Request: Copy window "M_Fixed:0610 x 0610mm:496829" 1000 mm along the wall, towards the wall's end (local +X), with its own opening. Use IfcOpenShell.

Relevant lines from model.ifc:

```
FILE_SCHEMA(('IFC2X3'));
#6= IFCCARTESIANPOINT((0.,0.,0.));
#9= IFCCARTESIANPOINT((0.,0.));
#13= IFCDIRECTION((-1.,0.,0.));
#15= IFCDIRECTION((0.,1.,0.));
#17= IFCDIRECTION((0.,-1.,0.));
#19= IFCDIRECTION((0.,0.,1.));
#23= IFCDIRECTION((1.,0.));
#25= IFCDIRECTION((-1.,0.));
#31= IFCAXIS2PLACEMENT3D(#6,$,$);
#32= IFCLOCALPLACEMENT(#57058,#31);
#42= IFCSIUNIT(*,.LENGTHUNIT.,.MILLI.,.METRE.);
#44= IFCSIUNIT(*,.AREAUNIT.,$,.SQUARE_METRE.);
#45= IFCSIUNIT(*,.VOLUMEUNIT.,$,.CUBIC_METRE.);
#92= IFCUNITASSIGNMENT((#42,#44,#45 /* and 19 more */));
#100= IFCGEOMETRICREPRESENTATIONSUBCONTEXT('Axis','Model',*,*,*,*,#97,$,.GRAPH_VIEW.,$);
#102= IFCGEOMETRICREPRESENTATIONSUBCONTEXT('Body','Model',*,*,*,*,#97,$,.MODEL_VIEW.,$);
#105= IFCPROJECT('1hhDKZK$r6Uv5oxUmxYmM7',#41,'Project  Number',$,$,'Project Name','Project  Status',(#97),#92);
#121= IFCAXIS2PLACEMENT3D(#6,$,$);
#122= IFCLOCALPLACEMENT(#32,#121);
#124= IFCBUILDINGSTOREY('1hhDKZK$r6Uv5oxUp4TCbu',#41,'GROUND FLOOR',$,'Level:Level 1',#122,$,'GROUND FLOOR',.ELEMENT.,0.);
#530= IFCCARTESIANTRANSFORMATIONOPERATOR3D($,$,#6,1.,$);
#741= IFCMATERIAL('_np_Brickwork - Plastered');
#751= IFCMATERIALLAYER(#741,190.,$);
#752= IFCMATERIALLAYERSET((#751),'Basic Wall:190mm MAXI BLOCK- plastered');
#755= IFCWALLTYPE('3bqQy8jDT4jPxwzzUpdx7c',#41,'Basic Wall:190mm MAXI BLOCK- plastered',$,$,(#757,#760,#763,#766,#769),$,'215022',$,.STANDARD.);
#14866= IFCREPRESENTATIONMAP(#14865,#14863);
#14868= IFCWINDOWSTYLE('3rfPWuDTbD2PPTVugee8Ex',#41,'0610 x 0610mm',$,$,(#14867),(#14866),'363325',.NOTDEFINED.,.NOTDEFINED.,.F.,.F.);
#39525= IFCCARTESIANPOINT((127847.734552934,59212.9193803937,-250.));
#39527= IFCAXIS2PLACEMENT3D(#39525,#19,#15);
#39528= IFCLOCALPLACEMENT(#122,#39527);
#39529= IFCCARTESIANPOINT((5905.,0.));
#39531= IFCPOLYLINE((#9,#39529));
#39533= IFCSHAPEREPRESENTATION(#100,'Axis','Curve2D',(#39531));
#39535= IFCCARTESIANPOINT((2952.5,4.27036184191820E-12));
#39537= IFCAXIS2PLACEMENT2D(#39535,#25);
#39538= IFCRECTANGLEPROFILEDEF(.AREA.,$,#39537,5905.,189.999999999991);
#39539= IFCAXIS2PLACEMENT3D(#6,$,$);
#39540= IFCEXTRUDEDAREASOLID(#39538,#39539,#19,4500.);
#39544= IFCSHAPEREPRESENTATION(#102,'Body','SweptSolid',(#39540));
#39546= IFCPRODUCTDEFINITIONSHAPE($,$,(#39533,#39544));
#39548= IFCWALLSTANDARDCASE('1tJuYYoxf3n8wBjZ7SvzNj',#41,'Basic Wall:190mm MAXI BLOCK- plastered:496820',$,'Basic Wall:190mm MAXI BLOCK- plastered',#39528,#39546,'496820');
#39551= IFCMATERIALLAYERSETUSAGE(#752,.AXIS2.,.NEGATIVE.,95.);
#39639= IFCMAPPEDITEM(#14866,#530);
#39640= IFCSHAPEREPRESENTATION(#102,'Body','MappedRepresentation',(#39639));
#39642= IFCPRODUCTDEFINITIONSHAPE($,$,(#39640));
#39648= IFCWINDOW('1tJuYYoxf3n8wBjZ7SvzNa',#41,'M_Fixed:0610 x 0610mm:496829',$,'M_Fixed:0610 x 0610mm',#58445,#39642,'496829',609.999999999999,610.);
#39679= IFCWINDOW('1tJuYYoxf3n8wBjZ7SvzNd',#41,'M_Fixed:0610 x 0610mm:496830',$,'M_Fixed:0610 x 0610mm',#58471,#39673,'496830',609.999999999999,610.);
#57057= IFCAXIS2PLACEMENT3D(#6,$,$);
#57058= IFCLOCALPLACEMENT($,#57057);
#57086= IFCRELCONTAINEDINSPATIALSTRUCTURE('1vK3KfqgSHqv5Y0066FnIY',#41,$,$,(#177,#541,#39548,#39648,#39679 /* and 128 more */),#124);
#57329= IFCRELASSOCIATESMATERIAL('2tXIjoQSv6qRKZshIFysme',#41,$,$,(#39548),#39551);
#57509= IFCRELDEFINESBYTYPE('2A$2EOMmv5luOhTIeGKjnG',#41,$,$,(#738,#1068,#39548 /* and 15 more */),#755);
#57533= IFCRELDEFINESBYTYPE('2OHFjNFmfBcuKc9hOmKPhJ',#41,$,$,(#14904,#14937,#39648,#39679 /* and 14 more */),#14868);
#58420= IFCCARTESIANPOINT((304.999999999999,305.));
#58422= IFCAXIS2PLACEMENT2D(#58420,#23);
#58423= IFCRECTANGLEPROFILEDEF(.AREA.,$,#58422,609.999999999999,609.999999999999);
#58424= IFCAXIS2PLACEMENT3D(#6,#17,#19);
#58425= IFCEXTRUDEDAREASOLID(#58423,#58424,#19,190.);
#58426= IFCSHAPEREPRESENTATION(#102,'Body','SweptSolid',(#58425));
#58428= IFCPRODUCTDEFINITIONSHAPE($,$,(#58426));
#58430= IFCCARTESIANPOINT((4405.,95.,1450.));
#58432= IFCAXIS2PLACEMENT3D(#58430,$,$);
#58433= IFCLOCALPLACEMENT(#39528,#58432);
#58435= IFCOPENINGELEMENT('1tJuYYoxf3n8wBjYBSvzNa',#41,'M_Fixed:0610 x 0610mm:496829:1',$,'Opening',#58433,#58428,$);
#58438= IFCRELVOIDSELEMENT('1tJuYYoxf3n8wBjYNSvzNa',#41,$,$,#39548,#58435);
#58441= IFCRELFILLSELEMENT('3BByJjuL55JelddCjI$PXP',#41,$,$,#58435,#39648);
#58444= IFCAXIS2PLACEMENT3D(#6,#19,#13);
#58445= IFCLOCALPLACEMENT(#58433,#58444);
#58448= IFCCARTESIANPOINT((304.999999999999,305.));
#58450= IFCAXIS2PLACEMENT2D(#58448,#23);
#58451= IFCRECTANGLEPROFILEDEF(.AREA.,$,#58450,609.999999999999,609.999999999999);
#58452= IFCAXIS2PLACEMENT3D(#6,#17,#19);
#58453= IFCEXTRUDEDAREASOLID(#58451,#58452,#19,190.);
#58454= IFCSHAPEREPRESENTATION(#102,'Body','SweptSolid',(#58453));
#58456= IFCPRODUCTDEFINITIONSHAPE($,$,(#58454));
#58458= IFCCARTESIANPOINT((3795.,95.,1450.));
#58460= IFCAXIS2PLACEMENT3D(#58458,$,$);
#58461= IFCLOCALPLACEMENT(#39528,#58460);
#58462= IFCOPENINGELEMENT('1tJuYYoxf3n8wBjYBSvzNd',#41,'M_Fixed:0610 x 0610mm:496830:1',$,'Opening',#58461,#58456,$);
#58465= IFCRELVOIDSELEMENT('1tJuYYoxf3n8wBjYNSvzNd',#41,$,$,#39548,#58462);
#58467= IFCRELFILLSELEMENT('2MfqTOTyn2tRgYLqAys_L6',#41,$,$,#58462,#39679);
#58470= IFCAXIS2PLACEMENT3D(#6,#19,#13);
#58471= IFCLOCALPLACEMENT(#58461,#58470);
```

```python
import ifcopenshell
import ifcopenshell.api.feature
import ifcopenshell.api.geometry
import ifcopenshell.api.root
import ifcopenshell.geom
import ifcopenshell.util.element
import ifcopenshell.util.placement
import ifcopenshell.util.shape
import ifcopenshell.util.unit

model = ifcopenshell.open("model.ifc")
unit_scale = ifcopenshell.util.unit.calculate_unit_scale(model)
settings = ifcopenshell.geom.settings()


def volume(element):
    """Net volume in cubic metres, openings subtracted."""
    shape = ifcopenshell.geom.create_shape(settings, element)
    return ifcopenshell.util.shape.get_volume(shape.geometry)


def reuse_history(source, copy):
    """copy_class also copies each property set's owner history, people and application; keep the originals."""
    for rel in copy.IsDefinedBy:
        if rel.is_a("IfcRelDefinesByProperties") and (history := rel.RelatingPropertyDefinition.OwnerHistory):
            rel.RelatingPropertyDefinition.OwnerHistory = source.OwnerHistory
            ifcopenshell.util.element.remove_deep2(model, history)


window = model.by_guid("1tJuYYoxf3n8wBjZ7SvzNa")
opening = window.FillsVoids[0].RelatingOpeningElement
wall = opening.VoidsElements[0].RelatingBuildingElement
before = volume(wall)
shift = ifcopenshell.util.placement.get_local_placement(wall.ObjectPlacement)[:3, 0] * 1 / unit_scale

# copy_class copies the void relationship, type, container and properties, but no geometry.
new_opening = ifcopenshell.api.root.copy_class(model, product=opening)
new_opening.Representation = ifcopenshell.util.element.copy_deep(
    model, opening.Representation, exclude=["IfcGeometricRepresentationContext", "IfcRepresentationMap"]
)
new_opening.Name = "M_Fixed:0610 x 0610mm"
new_window = ifcopenshell.api.root.copy_class(model, product=window)
new_window.Representation = ifcopenshell.util.element.copy_deep(
    model, window.Representation, exclude=["IfcGeometricRepresentationContext", "IfcRepresentationMap"]
)
new_window.Name = "M_Fixed:0610 x 0610mm"
new_window.Tag = None
reuse_history(window, new_window)
fills = ifcopenshell.api.feature.add_filling(model, opening=new_opening, element=new_window)
fills.OwnerHistory = new_window.OwnerHistory  # required in IFC2X3

for old, new in ((opening, new_opening), (window, new_window)):
    matrix = ifcopenshell.util.placement.get_local_placement(old.ObjectPlacement)
    matrix[:3, 3] += shift
    ifcopenshell.api.geometry.edit_object_placement(model, product=new, matrix=matrix, is_si=False)

after = volume(wall)

print(f"wall volume {before:.3f} -> {after:.3f} m3")

model.write("model_updated.ifc")
```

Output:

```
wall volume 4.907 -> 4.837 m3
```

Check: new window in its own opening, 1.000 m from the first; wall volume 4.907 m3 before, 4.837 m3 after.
